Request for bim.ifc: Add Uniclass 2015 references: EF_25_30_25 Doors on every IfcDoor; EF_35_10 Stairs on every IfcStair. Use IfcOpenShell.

First a look at what the model holds.

```python
import ifcopenshell

model = ifcopenshell.open("bim.ifc")
print(model.schema)
print("classifications:", [c.Name for c in model.by_type("IfcClassification")])
for ifc_class in ("IfcDoor", "IfcRoof", "IfcStair", "IfcWall", "IfcWindow"):
    print(ifc_class, len(model.by_type(ifc_class)))
```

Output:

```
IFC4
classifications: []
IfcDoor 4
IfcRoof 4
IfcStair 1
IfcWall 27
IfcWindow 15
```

```python
import ifcopenshell
import ifcopenshell.api.classification

model = ifcopenshell.open("bim.ifc")

system = ifcopenshell.api.classification.add_classification(model, classification="Uniclass 2015")

codes = {
    "IfcDoor": ("EF_25_30_25", "Doors"),
    "IfcStair": ("EF_35_10", "Stairs"),
}
for ifc_class, (code, name) in codes.items():
    products = model.by_type(ifc_class)
    ifcopenshell.api.classification.add_reference(
        model, products=products, classification=system, identification=code, name=name
    )
    print(code, len(products))

model.write("bim_edited.ifc")
```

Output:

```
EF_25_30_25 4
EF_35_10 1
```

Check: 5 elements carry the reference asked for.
